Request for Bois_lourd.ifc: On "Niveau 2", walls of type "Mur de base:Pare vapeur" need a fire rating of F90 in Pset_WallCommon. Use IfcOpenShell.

First a look at what the model holds.

```python
import ifcopenshell
import ifcopenshell.util.element

model = ifcopenshell.open("Bois_lourd.ifc")
print(model.schema)
storey = next(s for s in model.by_type("IfcBuildingStorey") if s.Name == "Niveau 2")
walls = [e for e in ifcopenshell.util.element.get_decomposition(storey) if e.is_a("IfcWall")]
seen = {}
for e in walls:
    element_type = ifcopenshell.util.element.get_type(e)
    key = (element_type.Name if element_type != e and element_type else None, ifcopenshell.util.element.get_pset(e, "Pset_WallCommon", "FireRating"))
    seen[key] = seen.get(key, 0) + 1
for (name, value), count in sorted(seen.items(), key=str):
    print(count, "x", name, "|", value)
```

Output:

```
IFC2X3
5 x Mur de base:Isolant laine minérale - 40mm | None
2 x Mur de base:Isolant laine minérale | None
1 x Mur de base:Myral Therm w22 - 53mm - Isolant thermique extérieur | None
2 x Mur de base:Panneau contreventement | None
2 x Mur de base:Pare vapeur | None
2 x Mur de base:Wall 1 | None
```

```python
import ifcopenshell
import ifcopenshell.api.pset
import ifcopenshell.util.element

model = ifcopenshell.open("Bois_lourd.ifc")

storey = next(s for s in model.by_type("IfcBuildingStorey") if s.Name == "Niveau 2")
walls = [e for e in ifcopenshell.util.element.get_decomposition(storey) if e.is_a("IfcWall")]

count = 0
for e in walls:
    element_type = ifcopenshell.util.element.get_type(e)
    if element_type in (None, e) or element_type.Name != "Mur de base:Pare vapeur":
        continue
    # add_pset returns the element's existing set when there is one.
    pset = ifcopenshell.api.pset.add_pset(model, product=e, name="Pset_WallCommon")
    ifcopenshell.api.pset.edit_pset(model, pset=pset, properties={"FireRating": "F90"})
    count += 1

print(count, "walls updated")

model.write("Bois_lourd_rev.ifc")
```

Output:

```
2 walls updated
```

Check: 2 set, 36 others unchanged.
